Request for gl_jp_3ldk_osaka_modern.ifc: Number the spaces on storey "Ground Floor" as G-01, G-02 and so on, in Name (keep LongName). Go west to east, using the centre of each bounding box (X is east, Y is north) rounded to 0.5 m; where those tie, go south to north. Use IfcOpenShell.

First a look at what the model holds.

```python
import ifcopenshell
import ifcopenshell.util.element
import ifcopenshell.util.placement

model = ifcopenshell.open("gl_jp_3ldk_osaka_modern.ifc")
print(model.schema)
storey = next(s for s in model.by_type("IfcBuildingStorey") if s.Name == "Ground Floor")
spaces = [e for e in ifcopenshell.util.element.get_decomposition(storey) if e.is_a("IfcSpace")]
for e in sorted(spaces, key=lambda e: e.id()):
    origin = ifcopenshell.util.placement.get_local_placement(e.ObjectPlacement)[:3, 3]
    print(e.id(), e.Name, e.LongName, origin.round(2) + 0.0, sep=" | ")
```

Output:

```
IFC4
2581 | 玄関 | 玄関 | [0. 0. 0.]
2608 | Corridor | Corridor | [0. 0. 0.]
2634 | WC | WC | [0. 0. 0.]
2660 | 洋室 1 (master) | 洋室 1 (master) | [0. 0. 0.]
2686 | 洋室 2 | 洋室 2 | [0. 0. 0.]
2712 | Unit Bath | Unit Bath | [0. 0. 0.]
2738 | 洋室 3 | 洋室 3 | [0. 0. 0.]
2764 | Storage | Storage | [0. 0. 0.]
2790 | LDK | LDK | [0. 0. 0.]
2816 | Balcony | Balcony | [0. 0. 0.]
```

```python
import ifcopenshell
import ifcopenshell.geom
import ifcopenshell.util.element
import ifcopenshell.util.shape

model = ifcopenshell.open("gl_jp_3ldk_osaka_modern.ifc")
settings = ifcopenshell.geom.settings()
settings.set("use-world-coords", True)


def centre(element):
    shape = ifcopenshell.geom.create_shape(settings, element)
    return ifcopenshell.util.shape.get_bbox_centroid(shape.geometry)


storey = next(s for s in model.by_type("IfcBuildingStorey") if s.Name == "Ground Floor")
spaces = [e for e in ifcopenshell.util.element.get_decomposition(storey) if e.is_a("IfcSpace")]

# Insertion points can sit at a corner or the storey origin, so sort by the geometry (in metres).
centres = {e: centre(e) for e in spaces}
spaces.sort(key=lambda e: (round(centres[e][0] / 0.5), centres[e][1]))

for i, e in enumerate(spaces, start=1):
    number = f"G-{i:02d}"
    e.Name = number
    print(e.id(), number)

model.write("gl_jp_3ldk_osaka_modern-out.ifc")
```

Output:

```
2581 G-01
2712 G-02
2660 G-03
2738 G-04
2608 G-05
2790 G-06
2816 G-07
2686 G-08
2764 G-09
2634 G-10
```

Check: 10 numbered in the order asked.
